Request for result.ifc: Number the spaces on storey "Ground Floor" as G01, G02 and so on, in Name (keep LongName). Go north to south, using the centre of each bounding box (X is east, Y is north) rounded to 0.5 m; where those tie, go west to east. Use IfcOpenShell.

First a look at what the model holds.

```python
import ifcopenshell
import ifcopenshell.util.element
import ifcopenshell.util.placement

model = ifcopenshell.open("result.ifc")
print(model.schema)
storey = next(s for s in model.by_type("IfcBuildingStorey") if s.Name == "Ground Floor")
spaces = [e for e in ifcopenshell.util.element.get_decomposition(storey) if e.is_a("IfcSpace")]
for e in sorted(spaces, key=lambda e: e.id()):
    origin = ifcopenshell.util.placement.get_local_placement(e.ObjectPlacement)[:3, 3]
    print(e.id(), e.Name, e.LongName, origin.round(2) + 0.0, sep=" | ")
```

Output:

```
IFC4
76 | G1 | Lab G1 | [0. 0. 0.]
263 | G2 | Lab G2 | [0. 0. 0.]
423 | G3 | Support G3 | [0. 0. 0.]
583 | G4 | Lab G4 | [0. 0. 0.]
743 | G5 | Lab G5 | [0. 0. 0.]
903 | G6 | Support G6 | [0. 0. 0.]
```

```python
import ifcopenshell
import ifcopenshell.geom
import ifcopenshell.util.element
import ifcopenshell.util.shape

model = ifcopenshell.open("result.ifc")
settings = ifcopenshell.geom.settings()
settings.set("use-world-coords", True)


def centre(element):
    shape = ifcopenshell.geom.create_shape(settings, element)
    return ifcopenshell.util.shape.get_bbox_centroid(shape.geometry)


storey = next(s for s in model.by_type("IfcBuildingStorey") if s.Name == "Ground Floor")
spaces = [e for e in ifcopenshell.util.element.get_decomposition(storey) if e.is_a("IfcSpace")]

# Insertion points can sit at a corner or the storey origin, so sort by the geometry (in metres).
centres = {e: centre(e) for e in spaces}
spaces.sort(key=lambda e: (-round(centres[e][1] / 0.5), centres[e][0]))

for i, e in enumerate(spaces, start=1):
    number = f"G{i:02d}"
    e.Name = number
    print(e.id(), number)

model.write("result_edited.ifc")
```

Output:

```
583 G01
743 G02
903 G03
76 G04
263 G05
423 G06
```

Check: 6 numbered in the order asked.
